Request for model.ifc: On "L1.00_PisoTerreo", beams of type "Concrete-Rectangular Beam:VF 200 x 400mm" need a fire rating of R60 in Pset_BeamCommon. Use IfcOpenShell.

First a look at what the model holds.

```python
import ifcopenshell
import ifcopenshell.util.element

model = ifcopenshell.open("model.ifc")
print(model.schema)
storey = next(s for s in model.by_type("IfcBuildingStorey") if s.Name == "L1.00_PisoTerreo")
beams = [e for e in ifcopenshell.util.element.get_decomposition(storey) if e.is_a("IfcBeam")]
seen = {}
for e in beams:
    element_type = ifcopenshell.util.element.get_type(e)
    key = (element_type.Name if element_type != e and element_type else None, ifcopenshell.util.element.get_pset(e, "Pset_BeamCommon", "FireRating"))
    seen[key] = seen.get(key, 0) + 1
for (name, value), count in sorted(seen.items(), key=str):
    print(count, "x", name, "|", value)
```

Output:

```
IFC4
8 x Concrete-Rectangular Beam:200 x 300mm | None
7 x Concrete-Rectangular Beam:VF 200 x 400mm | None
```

```python
import ifcopenshell
import ifcopenshell.api.pset
import ifcopenshell.util.element

model = ifcopenshell.open("model.ifc")

storey = next(s for s in model.by_type("IfcBuildingStorey") if s.Name == "L1.00_PisoTerreo")
beams = [e for e in ifcopenshell.util.element.get_decomposition(storey) if e.is_a("IfcBeam")]

count = 0
for e in beams:
    element_type = ifcopenshell.util.element.get_type(e)
    if element_type in (None, e) or element_type.Name != "Concrete-Rectangular Beam:VF 200 x 400mm":
        continue
    # add_pset returns the element's existing set when there is one.
    pset = ifcopenshell.api.pset.add_pset(model, product=e, name="Pset_BeamCommon")
    ifcopenshell.api.pset.edit_pset(model, pset=pset, properties={"FireRating": "R60"})
    count += 1

print(count, "beams updated")

model.write("model_edited.ifc")
```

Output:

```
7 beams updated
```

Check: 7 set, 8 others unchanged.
